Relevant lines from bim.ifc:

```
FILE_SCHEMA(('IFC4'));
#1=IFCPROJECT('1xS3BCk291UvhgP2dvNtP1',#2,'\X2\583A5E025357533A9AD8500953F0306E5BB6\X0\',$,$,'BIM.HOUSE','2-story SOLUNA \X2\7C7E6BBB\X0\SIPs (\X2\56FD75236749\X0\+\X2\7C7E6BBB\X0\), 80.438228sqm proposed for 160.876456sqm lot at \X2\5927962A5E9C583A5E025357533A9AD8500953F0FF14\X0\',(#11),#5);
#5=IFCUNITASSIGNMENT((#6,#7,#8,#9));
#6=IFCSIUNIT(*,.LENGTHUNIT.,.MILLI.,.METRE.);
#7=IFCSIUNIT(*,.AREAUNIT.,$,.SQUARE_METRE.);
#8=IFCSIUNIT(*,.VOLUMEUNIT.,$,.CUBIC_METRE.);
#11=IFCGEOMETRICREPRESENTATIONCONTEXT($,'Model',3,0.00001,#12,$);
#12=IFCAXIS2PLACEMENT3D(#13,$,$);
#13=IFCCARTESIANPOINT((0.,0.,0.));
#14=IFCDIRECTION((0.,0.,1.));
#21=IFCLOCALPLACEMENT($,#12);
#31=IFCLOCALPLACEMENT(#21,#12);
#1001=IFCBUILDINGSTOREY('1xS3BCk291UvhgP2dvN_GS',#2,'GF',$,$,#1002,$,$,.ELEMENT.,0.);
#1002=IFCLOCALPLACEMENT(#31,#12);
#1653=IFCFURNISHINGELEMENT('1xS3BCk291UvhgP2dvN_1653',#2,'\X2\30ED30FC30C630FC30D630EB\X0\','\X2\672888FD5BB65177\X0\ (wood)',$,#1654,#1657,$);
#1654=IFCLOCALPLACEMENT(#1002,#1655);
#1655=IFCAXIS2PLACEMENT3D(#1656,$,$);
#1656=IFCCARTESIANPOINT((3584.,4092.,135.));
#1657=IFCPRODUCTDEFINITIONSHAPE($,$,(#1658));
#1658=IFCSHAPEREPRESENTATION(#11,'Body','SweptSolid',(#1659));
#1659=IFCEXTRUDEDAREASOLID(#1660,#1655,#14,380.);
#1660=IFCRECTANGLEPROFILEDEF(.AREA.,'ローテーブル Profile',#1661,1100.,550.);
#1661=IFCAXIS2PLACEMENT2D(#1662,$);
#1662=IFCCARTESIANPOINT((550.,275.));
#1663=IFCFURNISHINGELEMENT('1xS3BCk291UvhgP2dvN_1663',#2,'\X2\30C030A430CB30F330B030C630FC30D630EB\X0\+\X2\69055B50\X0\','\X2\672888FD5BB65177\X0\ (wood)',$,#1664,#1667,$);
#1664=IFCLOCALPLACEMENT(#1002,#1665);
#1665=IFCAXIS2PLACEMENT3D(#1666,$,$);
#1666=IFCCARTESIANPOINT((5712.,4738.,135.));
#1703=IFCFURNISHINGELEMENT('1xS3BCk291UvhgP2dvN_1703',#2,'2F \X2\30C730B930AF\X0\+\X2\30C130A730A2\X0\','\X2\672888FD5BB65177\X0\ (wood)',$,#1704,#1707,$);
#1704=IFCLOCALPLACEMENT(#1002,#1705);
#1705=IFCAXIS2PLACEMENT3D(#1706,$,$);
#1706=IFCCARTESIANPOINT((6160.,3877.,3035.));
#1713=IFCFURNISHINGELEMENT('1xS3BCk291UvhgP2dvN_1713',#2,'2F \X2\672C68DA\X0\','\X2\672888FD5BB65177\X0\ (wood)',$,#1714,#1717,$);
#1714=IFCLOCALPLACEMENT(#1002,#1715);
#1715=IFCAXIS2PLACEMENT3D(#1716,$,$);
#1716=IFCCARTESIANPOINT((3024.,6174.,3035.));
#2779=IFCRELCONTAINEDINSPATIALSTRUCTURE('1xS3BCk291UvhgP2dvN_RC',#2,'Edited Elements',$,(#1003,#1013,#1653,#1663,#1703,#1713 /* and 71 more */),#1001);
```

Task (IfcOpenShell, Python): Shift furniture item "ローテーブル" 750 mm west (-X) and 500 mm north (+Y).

```python
import ifcopenshell
import ifcopenshell.api.geometry
import ifcopenshell.util.placement
import ifcopenshell.util.unit

model = ifcopenshell.open("bim.ifc")
unit_scale = ifcopenshell.util.unit.calculate_unit_scale(model)

item = model.by_guid("1xS3BCk291UvhgP2dvN_1653")
matrix = ifcopenshell.util.placement.get_local_placement(item.ObjectPlacement)
matrix[0, 3] -= 0.75 / unit_scale
matrix[1, 3] += 0.5 / unit_scale
ifcopenshell.api.geometry.edit_object_placement(model, product=item, matrix=matrix, is_si=False)

print(ifcopenshell.util.placement.get_local_placement(item.ObjectPlacement).round(3) + 0.0)

model.write("bim-out.ifc")
```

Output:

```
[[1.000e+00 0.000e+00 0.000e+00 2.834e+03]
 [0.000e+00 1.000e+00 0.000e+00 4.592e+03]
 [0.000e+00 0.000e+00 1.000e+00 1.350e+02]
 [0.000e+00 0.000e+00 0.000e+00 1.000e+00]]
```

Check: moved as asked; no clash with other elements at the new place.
